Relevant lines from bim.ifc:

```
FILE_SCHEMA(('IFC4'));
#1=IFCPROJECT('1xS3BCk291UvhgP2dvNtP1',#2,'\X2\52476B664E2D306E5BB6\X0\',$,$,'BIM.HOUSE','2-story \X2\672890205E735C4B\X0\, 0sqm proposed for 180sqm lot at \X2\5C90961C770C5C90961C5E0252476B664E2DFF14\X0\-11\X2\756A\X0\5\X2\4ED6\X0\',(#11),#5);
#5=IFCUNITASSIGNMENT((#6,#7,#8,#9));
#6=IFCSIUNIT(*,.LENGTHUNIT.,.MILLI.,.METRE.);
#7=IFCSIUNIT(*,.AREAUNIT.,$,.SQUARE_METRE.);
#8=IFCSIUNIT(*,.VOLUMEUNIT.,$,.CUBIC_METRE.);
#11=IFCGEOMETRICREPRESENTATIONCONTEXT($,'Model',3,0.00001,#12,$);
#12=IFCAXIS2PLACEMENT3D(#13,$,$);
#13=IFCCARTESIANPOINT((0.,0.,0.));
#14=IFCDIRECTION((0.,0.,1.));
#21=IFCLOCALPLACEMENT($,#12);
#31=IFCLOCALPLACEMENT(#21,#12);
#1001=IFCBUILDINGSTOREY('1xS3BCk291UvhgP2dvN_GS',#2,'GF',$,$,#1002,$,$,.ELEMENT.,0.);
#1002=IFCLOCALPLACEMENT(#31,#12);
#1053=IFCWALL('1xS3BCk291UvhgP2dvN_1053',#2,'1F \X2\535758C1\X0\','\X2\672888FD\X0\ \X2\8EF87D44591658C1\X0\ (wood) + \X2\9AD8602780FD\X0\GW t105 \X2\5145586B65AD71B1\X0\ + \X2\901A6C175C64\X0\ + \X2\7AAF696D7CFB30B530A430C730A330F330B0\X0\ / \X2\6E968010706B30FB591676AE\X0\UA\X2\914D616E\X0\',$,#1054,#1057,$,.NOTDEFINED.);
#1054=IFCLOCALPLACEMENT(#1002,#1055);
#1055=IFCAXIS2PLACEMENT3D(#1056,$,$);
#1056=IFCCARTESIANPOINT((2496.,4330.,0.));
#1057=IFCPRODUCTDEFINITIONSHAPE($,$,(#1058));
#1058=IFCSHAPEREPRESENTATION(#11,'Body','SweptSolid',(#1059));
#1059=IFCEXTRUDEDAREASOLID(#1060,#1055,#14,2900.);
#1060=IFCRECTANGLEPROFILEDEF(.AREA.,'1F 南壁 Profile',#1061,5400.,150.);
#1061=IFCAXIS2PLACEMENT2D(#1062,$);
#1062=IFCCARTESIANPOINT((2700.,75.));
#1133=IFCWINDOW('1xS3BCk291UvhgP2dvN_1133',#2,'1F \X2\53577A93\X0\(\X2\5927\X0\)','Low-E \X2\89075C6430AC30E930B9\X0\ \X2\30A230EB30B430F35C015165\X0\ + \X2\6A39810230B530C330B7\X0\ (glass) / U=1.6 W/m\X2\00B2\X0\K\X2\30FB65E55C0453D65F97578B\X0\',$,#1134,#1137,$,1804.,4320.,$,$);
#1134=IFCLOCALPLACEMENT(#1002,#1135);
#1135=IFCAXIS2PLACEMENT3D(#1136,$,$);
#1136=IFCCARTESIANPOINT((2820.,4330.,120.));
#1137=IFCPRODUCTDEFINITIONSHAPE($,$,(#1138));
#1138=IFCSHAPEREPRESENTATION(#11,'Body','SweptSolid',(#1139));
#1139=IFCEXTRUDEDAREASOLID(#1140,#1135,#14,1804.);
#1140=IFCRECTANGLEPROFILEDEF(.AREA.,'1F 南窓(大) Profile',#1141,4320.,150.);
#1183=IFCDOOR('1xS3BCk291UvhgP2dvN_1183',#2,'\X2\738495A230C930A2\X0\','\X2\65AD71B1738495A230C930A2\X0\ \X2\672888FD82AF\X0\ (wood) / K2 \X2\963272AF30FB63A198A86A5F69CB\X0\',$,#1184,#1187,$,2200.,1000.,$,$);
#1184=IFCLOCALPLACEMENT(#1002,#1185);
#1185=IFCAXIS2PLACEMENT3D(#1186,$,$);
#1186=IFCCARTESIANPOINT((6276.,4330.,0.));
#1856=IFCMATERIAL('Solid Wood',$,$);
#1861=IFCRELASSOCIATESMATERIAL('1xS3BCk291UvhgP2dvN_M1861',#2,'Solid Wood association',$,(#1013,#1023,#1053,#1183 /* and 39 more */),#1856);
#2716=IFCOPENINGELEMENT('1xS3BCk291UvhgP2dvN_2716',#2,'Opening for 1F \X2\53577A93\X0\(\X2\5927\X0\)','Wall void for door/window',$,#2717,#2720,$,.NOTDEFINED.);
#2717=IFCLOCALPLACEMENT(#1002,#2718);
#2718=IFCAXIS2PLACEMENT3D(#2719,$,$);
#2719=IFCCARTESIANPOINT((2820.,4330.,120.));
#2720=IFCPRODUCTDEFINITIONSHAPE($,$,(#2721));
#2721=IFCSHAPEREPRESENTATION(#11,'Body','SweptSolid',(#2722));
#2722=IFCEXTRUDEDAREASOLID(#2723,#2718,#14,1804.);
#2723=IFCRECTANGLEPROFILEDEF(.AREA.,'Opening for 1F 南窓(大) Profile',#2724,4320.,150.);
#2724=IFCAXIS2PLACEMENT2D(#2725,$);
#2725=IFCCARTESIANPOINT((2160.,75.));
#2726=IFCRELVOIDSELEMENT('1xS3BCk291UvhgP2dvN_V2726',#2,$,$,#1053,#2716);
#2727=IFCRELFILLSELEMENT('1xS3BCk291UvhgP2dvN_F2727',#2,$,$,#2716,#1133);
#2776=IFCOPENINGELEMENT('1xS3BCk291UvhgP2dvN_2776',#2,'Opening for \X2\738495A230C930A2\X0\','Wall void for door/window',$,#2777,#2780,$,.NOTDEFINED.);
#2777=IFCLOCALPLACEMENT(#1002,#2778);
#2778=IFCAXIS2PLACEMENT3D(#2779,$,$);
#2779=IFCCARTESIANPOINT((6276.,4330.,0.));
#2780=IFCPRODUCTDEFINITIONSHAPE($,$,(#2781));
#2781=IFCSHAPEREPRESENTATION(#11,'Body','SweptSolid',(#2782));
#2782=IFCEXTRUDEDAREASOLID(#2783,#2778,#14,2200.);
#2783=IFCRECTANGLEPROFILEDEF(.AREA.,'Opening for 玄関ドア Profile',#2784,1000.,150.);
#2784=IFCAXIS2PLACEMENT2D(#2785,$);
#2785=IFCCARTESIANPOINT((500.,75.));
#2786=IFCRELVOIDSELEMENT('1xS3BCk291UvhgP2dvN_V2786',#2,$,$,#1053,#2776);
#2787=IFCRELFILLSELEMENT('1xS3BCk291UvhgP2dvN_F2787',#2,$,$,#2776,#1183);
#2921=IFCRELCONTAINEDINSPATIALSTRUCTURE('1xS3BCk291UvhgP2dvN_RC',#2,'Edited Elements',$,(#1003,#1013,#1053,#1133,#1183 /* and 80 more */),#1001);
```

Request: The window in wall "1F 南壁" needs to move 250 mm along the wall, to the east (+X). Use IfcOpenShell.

```python
import ifcopenshell
import ifcopenshell.api.geometry
import ifcopenshell.util.placement

model = ifcopenshell.open("bim.ifc")

window = model.by_guid("1xS3BCk291UvhgP2dvN_1133")
opening = window.FillsVoids[0].RelatingOpeningElement
wall = opening.VoidsElements[0].RelatingBuildingElement

wall_matrix = ifcopenshell.util.placement.get_local_placement(wall.ObjectPlacement)
shift = wall_matrix[:3, 0] * 250.0
before = ifcopenshell.util.placement.get_local_placement(window.ObjectPlacement)[:3, 3].copy()

# The window is not placed relative to its opening, so move both.
for product in (opening, window):
    matrix = ifcopenshell.util.placement.get_local_placement(product.ObjectPlacement)
    matrix[:3, 3] += shift
    ifcopenshell.api.geometry.edit_object_placement(model, product=product, matrix=matrix, is_si=False)

after = ifcopenshell.util.placement.get_local_placement(window.ObjectPlacement)[:3, 3]
print("window moved by", (after - before).round(3) + 0.0)

model.write("bim_rev.ifc")
```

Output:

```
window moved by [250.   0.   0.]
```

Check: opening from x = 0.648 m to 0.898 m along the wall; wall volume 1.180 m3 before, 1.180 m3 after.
